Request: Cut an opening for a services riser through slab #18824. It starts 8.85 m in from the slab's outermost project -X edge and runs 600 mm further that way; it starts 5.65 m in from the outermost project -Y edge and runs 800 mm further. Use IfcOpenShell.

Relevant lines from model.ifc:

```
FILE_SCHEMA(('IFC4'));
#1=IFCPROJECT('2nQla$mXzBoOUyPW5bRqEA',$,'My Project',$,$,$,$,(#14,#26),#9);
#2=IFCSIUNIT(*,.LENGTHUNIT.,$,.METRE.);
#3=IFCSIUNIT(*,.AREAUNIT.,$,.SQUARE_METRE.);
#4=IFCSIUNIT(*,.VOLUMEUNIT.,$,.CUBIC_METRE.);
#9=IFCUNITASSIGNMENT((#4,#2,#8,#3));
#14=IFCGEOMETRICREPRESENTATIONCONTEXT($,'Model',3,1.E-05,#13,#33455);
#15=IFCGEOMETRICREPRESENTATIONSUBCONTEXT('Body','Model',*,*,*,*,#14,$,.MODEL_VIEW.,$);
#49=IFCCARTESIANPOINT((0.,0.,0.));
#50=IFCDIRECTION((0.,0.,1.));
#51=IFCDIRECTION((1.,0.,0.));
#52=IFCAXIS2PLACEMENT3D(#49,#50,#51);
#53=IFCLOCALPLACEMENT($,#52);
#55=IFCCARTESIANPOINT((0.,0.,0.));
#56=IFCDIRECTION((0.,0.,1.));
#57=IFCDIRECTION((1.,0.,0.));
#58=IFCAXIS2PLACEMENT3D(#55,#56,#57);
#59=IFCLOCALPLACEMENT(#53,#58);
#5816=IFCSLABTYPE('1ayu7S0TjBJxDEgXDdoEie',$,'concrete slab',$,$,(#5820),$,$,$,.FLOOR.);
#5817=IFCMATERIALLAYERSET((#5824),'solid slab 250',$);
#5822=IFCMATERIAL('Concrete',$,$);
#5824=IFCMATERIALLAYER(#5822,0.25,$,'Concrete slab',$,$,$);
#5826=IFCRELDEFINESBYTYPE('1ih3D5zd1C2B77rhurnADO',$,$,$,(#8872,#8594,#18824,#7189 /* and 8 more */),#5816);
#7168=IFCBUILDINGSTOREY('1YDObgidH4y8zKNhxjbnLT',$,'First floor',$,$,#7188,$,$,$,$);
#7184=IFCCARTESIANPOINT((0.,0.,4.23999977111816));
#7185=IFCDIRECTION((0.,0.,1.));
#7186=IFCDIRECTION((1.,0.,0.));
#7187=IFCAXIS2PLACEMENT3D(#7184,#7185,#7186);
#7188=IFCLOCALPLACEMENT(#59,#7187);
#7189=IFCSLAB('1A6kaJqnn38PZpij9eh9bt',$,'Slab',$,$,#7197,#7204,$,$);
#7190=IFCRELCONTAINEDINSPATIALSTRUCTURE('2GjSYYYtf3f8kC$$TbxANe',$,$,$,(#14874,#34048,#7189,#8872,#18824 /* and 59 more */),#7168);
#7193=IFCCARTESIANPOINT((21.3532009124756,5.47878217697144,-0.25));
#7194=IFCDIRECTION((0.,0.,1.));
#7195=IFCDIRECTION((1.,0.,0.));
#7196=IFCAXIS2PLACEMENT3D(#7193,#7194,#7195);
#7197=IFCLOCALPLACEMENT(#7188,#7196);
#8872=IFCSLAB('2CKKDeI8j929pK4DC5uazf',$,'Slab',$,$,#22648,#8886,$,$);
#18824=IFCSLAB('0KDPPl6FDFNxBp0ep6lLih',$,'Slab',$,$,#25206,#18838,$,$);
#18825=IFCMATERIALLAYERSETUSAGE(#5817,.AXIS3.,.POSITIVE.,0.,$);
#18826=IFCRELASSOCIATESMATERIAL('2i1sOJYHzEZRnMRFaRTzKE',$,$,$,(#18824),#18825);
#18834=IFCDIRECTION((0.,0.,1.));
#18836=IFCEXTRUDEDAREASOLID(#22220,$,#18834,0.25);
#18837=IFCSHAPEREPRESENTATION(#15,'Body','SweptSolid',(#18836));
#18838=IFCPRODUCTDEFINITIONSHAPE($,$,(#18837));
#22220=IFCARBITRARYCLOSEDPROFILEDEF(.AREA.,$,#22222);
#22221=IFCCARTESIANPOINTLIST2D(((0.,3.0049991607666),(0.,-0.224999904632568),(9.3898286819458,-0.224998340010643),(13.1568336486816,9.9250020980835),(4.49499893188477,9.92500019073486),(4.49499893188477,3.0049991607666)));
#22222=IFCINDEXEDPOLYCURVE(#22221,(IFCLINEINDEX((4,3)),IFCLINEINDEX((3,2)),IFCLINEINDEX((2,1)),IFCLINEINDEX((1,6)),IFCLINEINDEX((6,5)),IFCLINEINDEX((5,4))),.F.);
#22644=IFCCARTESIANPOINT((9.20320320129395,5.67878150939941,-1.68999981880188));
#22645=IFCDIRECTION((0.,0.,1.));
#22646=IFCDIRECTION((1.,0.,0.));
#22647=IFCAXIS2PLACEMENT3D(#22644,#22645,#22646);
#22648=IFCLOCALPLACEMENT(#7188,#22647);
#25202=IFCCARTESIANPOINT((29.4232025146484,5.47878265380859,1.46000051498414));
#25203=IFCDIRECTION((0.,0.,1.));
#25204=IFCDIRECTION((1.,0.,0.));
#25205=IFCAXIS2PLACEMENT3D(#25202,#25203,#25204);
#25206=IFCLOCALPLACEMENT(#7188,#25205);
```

```python
import numpy as np
import ifcopenshell
import ifcopenshell.api.feature
import ifcopenshell.api.geometry
import ifcopenshell.api.root
import ifcopenshell.geom
import ifcopenshell.util.placement
import ifcopenshell.util.representation
import ifcopenshell.util.shape
import ifcopenshell.util.unit

model = ifcopenshell.open("model.ifc")
unit_scale = ifcopenshell.util.unit.calculate_unit_scale(model)
settings = ifcopenshell.geom.settings()


def volume(element):
    """Net volume in cubic metres, openings subtracted."""
    shape = ifcopenshell.geom.create_shape(settings, element)
    return ifcopenshell.util.shape.get_volume(shape.geometry)


slab = model.by_guid("0KDPPl6FDFNxBp0ep6lLih")
before = volume(slab)

# Extent in the slab's own axes, in metres. The edges named are its -X and -Y sides.
slab_shape = ifcopenshell.geom.create_shape(settings, slab)
vertices = ifcopenshell.util.shape.get_vertices(slab_shape.geometry)
x_min, y_min, bottom = vertices.min(axis=0)
top = vertices[:, 2].max()

opening = ifcopenshell.api.root.create_entity(model, ifc_class="IfcOpeningElement", name="Services riser opening", predefined_type="OPENING")
context = ifcopenshell.util.representation.get_context(model, "Model", "Body", "MODEL_VIEW")
width, depth = 0.6, 0.8
outline = [(0.0, 0.0), (width, 0.0), (width, depth), (0.0, depth), (0.0, 0.0)]
# Overshoot both faces by 50 mm so the cut is clean.
shape = ifcopenshell.api.geometry.add_slab_representation(
    model, context=context, depth=top - bottom + 0.1, polyline=outline
)
ifcopenshell.api.geometry.assign_representation(model, product=opening, representation=shape)

matrix = ifcopenshell.util.placement.get_local_placement(slab.ObjectPlacement)
matrix[:, 3] = matrix @ np.append(np.array([x_min + 8.85, y_min + 5.65, bottom - 0.05]) / unit_scale, 1.0)
ifcopenshell.api.geometry.edit_object_placement(model, product=opening, matrix=matrix, is_si=False)
ifcopenshell.api.feature.add_feature(model, feature=opening, element=slab)

after = volume(slab)

print(f"slab volume {before:.3f} -> {after:.3f} m3")

model.write("model_edited.ifc")
```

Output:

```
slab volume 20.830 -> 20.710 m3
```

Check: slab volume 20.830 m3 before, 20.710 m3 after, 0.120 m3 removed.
